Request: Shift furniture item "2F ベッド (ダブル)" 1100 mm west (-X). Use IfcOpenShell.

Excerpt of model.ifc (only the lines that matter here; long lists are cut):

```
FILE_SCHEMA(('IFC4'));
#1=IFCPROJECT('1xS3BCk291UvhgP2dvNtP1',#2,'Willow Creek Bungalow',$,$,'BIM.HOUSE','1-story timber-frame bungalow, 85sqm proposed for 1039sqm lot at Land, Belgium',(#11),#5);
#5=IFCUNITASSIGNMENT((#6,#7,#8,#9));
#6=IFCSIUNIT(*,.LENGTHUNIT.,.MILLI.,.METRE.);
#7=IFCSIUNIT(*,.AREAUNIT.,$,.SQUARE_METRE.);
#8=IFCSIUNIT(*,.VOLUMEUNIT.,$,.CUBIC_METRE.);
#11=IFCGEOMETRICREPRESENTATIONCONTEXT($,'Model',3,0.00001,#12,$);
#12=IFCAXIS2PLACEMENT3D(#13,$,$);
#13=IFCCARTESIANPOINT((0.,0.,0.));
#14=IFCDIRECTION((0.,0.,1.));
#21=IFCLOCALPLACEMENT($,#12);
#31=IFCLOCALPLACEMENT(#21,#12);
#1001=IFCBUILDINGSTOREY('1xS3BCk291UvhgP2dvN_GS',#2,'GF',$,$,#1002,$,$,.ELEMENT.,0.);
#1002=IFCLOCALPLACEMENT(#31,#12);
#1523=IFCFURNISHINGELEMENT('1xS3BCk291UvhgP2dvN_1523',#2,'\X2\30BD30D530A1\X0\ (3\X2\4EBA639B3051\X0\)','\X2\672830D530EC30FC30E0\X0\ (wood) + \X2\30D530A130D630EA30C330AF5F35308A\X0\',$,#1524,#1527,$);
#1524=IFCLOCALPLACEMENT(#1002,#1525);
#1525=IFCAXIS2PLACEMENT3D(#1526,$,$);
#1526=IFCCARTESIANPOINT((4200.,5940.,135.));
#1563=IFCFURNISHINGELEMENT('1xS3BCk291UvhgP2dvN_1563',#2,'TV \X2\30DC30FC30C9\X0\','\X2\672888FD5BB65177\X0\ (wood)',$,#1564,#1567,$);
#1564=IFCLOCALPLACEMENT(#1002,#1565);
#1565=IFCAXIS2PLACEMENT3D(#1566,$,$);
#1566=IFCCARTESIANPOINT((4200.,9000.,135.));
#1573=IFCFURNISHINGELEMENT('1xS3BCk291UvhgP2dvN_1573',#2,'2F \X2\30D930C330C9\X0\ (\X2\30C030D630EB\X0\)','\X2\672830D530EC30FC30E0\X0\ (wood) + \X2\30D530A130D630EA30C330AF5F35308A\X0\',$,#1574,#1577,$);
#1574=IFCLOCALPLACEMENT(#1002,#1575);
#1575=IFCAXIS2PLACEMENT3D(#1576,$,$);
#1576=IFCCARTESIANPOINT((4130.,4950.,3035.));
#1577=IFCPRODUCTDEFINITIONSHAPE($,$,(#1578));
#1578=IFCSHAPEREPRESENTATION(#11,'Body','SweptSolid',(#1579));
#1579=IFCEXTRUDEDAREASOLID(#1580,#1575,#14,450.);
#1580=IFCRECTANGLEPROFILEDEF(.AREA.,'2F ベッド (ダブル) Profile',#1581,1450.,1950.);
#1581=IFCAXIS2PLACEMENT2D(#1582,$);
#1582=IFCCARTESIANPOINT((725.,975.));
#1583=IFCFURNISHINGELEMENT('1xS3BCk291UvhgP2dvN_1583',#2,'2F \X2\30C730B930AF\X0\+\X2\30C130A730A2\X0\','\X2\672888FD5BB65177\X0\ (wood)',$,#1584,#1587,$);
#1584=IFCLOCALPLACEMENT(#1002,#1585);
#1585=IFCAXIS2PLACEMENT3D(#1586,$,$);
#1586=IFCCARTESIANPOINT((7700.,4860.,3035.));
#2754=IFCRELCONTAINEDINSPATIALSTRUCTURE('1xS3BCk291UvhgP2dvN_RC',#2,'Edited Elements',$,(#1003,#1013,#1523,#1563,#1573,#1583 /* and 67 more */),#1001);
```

```python
import ifcopenshell
import ifcopenshell.api.geometry
import ifcopenshell.util.placement
import ifcopenshell.util.unit

model = ifcopenshell.open("model.ifc")
unit_scale = ifcopenshell.util.unit.calculate_unit_scale(model)

item = model.by_guid("1xS3BCk291UvhgP2dvN_1573")
matrix = ifcopenshell.util.placement.get_local_placement(item.ObjectPlacement)
matrix[0, 3] -= 1.1 / unit_scale
ifcopenshell.api.geometry.edit_object_placement(model, product=item, matrix=matrix, is_si=False)

print(ifcopenshell.util.placement.get_local_placement(item.ObjectPlacement).round(3) + 0.0)

model.write("model_rev.ifc")
```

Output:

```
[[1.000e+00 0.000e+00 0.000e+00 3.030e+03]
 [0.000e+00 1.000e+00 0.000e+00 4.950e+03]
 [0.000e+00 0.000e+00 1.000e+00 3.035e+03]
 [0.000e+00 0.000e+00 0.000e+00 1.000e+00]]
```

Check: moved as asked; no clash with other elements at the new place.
